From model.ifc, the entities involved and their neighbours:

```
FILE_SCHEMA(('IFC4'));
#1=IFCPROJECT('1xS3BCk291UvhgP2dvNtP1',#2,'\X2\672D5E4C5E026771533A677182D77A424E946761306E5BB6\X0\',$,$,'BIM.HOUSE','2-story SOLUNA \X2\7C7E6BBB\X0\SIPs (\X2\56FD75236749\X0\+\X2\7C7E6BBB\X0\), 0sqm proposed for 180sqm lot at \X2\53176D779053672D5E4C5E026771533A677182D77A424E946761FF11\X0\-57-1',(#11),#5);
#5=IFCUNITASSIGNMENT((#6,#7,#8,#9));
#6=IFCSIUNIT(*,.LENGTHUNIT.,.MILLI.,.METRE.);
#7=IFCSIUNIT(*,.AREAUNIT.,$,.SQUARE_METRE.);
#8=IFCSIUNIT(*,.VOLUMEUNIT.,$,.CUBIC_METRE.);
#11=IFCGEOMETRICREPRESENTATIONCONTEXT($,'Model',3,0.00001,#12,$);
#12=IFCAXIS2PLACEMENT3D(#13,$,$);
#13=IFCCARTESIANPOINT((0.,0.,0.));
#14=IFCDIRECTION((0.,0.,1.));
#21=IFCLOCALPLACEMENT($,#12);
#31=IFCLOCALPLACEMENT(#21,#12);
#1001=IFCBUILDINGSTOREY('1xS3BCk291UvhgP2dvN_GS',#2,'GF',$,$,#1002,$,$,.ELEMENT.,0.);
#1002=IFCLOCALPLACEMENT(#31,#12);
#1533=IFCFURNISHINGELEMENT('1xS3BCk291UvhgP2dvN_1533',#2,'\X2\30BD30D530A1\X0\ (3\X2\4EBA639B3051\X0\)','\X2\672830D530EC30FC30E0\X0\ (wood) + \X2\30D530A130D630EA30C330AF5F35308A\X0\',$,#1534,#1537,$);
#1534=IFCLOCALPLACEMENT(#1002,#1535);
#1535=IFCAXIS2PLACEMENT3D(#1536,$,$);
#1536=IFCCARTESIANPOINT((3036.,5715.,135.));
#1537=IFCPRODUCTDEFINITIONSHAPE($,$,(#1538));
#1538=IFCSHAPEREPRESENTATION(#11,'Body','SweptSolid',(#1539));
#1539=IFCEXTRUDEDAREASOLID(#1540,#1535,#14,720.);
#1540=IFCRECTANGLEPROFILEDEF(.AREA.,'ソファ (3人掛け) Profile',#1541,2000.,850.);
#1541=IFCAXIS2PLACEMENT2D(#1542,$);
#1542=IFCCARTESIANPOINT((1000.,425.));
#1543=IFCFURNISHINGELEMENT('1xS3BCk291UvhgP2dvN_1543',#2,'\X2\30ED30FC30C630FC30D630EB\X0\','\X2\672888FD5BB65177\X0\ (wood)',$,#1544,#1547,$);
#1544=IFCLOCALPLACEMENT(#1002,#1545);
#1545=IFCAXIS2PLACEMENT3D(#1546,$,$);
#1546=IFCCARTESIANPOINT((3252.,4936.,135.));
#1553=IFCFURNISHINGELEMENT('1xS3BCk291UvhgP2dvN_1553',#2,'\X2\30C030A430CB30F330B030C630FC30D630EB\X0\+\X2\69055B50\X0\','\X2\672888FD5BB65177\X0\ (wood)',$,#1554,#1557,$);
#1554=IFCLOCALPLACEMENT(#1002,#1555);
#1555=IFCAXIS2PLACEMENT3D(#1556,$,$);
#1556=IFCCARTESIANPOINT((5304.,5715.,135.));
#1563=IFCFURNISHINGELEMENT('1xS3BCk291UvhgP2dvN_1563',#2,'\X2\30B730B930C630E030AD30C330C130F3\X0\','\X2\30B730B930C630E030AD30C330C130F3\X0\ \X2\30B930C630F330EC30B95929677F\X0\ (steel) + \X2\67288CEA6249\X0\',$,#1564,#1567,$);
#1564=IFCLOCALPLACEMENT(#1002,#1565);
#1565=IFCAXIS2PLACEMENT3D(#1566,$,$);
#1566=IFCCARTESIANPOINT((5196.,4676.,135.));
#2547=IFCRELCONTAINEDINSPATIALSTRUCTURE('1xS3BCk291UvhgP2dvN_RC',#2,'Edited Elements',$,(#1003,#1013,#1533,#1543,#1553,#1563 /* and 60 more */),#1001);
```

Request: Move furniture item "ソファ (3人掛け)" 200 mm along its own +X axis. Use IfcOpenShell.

```python
import ifcopenshell
import ifcopenshell.api.geometry
import ifcopenshell.util.placement
import ifcopenshell.util.unit

model = ifcopenshell.open("model.ifc")
unit_scale = ifcopenshell.util.unit.calculate_unit_scale(model)

item = model.by_guid("1xS3BCk291UvhgP2dvN_1533")
matrix = ifcopenshell.util.placement.get_local_placement(item.ObjectPlacement)
matrix[:3, 3] += matrix[:3, 0] * 0.2 / unit_scale
ifcopenshell.api.geometry.edit_object_placement(model, product=item, matrix=matrix, is_si=False)

print(ifcopenshell.util.placement.get_local_placement(item.ObjectPlacement).round(3) + 0.0)

model.write("model_v2.ifc")
```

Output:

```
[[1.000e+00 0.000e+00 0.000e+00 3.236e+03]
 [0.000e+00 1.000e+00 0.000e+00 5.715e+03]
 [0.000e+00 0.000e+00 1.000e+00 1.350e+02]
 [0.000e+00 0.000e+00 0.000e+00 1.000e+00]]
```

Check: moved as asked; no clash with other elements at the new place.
